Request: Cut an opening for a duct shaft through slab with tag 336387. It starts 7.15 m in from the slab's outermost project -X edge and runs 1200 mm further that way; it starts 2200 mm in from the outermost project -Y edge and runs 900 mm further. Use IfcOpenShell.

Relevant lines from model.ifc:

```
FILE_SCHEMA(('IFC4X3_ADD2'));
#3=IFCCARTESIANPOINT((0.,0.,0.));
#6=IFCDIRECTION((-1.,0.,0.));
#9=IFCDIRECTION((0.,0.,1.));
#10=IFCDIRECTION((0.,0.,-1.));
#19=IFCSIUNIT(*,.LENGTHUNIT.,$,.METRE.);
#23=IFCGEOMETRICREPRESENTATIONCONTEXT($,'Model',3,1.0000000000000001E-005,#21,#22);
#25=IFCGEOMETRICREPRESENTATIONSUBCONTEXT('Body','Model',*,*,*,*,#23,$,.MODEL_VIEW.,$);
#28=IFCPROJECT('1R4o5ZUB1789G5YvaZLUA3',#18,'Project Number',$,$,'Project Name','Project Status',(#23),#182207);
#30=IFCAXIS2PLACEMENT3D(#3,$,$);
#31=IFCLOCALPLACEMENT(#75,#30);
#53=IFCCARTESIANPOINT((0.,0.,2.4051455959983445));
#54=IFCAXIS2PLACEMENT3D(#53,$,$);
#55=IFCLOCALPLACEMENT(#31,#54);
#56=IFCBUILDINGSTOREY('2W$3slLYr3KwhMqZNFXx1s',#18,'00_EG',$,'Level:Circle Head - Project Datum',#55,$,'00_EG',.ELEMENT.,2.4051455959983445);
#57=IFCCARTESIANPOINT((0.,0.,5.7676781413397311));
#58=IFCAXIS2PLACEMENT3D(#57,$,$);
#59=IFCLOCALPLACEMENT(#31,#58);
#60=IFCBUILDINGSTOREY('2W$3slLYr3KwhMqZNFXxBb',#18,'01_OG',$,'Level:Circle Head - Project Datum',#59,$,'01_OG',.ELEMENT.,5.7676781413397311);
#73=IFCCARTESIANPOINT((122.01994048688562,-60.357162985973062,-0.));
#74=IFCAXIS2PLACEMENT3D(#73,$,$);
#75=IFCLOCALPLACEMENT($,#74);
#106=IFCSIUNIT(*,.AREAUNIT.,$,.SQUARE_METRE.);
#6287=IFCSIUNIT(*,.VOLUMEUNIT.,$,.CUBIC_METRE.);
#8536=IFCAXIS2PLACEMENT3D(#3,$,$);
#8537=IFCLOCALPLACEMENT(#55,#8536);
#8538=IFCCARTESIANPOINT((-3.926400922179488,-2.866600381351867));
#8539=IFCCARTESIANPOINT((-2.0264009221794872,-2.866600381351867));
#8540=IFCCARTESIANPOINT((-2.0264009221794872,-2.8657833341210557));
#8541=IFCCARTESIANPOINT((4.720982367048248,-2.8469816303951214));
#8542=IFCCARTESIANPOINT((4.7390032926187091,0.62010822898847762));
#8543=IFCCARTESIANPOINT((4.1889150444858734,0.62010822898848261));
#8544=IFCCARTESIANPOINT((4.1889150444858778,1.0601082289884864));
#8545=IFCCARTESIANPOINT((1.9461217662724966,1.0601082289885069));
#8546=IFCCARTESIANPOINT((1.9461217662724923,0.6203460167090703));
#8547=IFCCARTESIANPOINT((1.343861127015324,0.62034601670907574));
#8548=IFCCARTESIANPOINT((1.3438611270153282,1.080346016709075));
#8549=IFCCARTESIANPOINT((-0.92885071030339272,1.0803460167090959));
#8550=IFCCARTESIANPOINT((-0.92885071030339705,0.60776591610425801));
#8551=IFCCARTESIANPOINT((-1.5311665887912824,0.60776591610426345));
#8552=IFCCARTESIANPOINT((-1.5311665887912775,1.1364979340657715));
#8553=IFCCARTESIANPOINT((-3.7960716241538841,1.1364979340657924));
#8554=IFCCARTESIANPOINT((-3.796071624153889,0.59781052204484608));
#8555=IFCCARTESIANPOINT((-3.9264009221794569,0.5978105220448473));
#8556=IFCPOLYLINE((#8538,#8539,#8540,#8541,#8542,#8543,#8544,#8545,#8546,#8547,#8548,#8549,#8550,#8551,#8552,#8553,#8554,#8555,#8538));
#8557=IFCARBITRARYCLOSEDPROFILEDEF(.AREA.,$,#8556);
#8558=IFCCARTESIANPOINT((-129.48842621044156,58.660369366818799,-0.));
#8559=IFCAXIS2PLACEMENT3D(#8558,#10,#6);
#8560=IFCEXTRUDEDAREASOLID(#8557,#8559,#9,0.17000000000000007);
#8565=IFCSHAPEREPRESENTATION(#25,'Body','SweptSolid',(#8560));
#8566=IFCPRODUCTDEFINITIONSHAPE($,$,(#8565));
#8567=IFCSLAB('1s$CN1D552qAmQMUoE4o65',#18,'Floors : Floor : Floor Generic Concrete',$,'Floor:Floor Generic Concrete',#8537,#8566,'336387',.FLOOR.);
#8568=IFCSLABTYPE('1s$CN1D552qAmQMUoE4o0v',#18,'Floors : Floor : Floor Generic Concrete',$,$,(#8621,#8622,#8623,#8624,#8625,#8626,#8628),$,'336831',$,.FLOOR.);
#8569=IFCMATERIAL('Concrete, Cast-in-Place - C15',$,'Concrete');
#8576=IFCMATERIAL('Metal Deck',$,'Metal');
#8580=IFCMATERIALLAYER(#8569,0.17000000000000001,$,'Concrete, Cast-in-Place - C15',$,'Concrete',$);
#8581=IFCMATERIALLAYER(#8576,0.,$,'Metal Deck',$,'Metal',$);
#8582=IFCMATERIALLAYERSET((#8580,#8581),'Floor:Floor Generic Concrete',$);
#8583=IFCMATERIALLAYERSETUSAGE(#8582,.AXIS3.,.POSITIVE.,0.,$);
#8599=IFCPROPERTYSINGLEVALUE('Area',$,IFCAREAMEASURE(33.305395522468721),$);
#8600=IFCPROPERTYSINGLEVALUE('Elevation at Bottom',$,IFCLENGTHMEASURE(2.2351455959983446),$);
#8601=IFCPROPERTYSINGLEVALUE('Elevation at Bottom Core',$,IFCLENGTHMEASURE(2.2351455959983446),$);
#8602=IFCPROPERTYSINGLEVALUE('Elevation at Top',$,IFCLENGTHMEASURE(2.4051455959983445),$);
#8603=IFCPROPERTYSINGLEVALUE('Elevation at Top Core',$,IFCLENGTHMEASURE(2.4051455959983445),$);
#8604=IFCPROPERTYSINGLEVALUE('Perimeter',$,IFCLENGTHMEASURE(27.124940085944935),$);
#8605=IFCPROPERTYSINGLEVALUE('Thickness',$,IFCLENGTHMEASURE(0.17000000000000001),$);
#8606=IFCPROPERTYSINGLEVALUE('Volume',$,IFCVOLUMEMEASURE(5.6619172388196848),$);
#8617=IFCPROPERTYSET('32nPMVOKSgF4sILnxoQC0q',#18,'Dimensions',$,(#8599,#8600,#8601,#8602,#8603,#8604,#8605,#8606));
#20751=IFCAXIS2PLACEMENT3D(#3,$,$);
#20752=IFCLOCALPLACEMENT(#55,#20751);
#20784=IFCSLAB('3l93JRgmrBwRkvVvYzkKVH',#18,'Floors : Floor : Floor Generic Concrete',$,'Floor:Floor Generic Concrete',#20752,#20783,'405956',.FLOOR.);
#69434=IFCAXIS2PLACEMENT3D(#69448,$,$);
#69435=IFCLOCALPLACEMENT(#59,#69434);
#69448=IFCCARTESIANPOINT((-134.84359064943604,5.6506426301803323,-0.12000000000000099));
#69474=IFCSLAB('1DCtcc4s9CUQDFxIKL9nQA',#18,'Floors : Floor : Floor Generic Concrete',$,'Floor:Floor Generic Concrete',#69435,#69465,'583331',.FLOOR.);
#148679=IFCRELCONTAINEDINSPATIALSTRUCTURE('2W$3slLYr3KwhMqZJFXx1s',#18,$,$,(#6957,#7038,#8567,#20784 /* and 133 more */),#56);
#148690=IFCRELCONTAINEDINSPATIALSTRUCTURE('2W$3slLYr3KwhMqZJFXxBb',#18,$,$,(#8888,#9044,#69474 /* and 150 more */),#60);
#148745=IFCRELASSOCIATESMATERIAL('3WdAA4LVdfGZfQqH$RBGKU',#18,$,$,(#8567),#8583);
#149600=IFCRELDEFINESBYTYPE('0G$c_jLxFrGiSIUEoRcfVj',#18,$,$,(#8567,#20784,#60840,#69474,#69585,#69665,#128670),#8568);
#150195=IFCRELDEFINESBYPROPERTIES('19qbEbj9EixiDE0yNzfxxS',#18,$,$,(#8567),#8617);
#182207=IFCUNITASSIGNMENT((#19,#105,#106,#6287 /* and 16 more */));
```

```python
import numpy as np
import ifcopenshell
import ifcopenshell.api.feature
import ifcopenshell.api.geometry
import ifcopenshell.api.pset
import ifcopenshell.api.root
import ifcopenshell.geom
import ifcopenshell.util.element
import ifcopenshell.util.placement
import ifcopenshell.util.representation
import ifcopenshell.util.shape
import ifcopenshell.util.unit

model = ifcopenshell.open("model.ifc")
unit_scale = ifcopenshell.util.unit.calculate_unit_scale(model)
area_scale = ifcopenshell.util.unit.calculate_unit_scale(model, "AREAUNIT")
volume_scale = ifcopenshell.util.unit.calculate_unit_scale(model, "VOLUMEUNIT")
settings = ifcopenshell.geom.settings()


def volume(element):
    """Net volume in cubic metres, openings subtracted."""
    shape = ifcopenshell.geom.create_shape(settings, element)
    return ifcopenshell.util.shape.get_volume(shape.geometry)


slab = model.by_guid("1s$CN1D552qAmQMUoE4o65")
before = volume(slab)

# Extent in the slab's own axes, in metres. The edges named are its -X and -Y sides.
slab_shape = ifcopenshell.geom.create_shape(settings, slab)
vertices = ifcopenshell.util.shape.get_vertices(slab_shape.geometry)
x_min, y_min, bottom = vertices.min(axis=0)
top = vertices[:, 2].max()

opening = ifcopenshell.api.root.create_entity(model, ifc_class="IfcOpeningElement", name="Duct shaft opening", predefined_type="OPENING")
context = ifcopenshell.util.representation.get_context(model, "Model", "Body", "MODEL_VIEW")
width, depth = 1.2, 0.9
outline = [(0.0, 0.0), (width, 0.0), (width, depth), (0.0, depth), (0.0, 0.0)]
# Overshoot both faces by 50 mm so the cut is clean.
shape = ifcopenshell.api.geometry.add_slab_representation(
    model, context=context, depth=top - bottom + 0.1, polyline=outline
)
ifcopenshell.api.geometry.assign_representation(model, product=opening, representation=shape)

matrix = ifcopenshell.util.placement.get_local_placement(slab.ObjectPlacement)
matrix[:, 3] = matrix @ np.append(np.array([x_min + 7.15, y_min + 2.2, bottom - 0.05]) / unit_scale, 1.0)
ifcopenshell.api.geometry.edit_object_placement(model, product=opening, matrix=matrix, is_si=False)
ifcopenshell.api.feature.add_feature(model, feature=opening, element=slab)

after = volume(slab)

# Update the slab's stored quantities.
pset = model.by_id(ifcopenshell.util.element.get_pset(slab, "Dimensions", should_inherit=False)["id"])
ifcopenshell.api.pset.edit_pset(model, pset=pset, properties={
    "Area": model.create_entity("IfcAreaMeasure", after / (top - bottom) / area_scale),
    "Volume": model.create_entity("IfcVolumeMeasure", after / volume_scale),
})

print(f"slab volume {before:.3f} -> {after:.3f} m3")

model.write("model_updated.ifc")
```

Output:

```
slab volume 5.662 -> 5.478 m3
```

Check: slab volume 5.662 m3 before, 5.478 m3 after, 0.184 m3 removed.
